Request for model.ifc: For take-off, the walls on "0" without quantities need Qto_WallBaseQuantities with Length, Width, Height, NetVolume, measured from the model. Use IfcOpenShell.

First a look at what the model holds.

```python
import ifcopenshell
import ifcopenshell.util.element
import ifcopenshell.util.unit

model = ifcopenshell.open("model.ifc")
print(model.schema)
for unit_type in ("LENGTHUNIT", "AREAUNIT", "VOLUMEUNIT"):
    print(unit_type, ifcopenshell.util.unit.calculate_unit_scale(model, unit_type))
storey = next(s for s in model.by_type("IfcBuildingStorey") if s.Name == "0")
walls = [e for e in ifcopenshell.util.element.get_decomposition(storey) if e.is_a("IfcWall")]
for e in sorted(walls, key=lambda e: e.id()):
    print(e.id(), e.is_a(), e.Name, list(ifcopenshell.util.element.get_psets(e, qtos_only=True)), sep=" | ")
```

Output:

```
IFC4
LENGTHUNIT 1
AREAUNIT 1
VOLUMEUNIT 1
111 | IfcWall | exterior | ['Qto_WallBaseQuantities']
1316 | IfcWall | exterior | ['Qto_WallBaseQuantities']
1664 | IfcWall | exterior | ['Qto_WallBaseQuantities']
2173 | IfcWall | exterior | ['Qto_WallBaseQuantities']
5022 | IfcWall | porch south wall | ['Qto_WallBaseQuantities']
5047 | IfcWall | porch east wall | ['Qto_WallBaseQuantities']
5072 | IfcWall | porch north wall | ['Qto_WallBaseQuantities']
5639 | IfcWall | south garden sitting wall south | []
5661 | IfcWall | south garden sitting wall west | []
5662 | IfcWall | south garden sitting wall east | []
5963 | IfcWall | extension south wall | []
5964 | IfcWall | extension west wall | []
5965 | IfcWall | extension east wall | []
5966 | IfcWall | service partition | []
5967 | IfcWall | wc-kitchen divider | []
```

```python
import ifcopenshell
import ifcopenshell.api.pset
import ifcopenshell.geom
import ifcopenshell.util.element
import ifcopenshell.util.shape
import ifcopenshell.util.unit

model = ifcopenshell.open("model.ifc")
unit_scale = ifcopenshell.util.unit.calculate_unit_scale(model)
volume_scale = ifcopenshell.util.unit.calculate_unit_scale(model, "VOLUMEUNIT")
settings = ifcopenshell.geom.settings()

storey = next(s for s in model.by_type("IfcBuildingStorey") if s.Name == "0")
walls = [e for e in ifcopenshell.util.element.get_decomposition(storey) if e.is_a("IfcWall")]

for e in sorted(walls, key=lambda e: e.id()):
    if ifcopenshell.util.element.get_psets(e, qtos_only=True, should_inherit=False):
        continue
    # Geometry comes back in metres, in the element's own axes.
    shape = ifcopenshell.geom.create_shape(settings, e)
    values = {
        "Length": ifcopenshell.util.shape.get_x(shape.geometry) / unit_scale,
        "Width": ifcopenshell.util.shape.get_y(shape.geometry) / unit_scale,
        "Height": ifcopenshell.util.shape.get_z(shape.geometry) / unit_scale,
        "NetVolume": ifcopenshell.util.shape.get_volume(shape.geometry) / volume_scale,
    }
    qto = ifcopenshell.api.pset.add_qto(model, product=e, name="Qto_WallBaseQuantities")
    ifcopenshell.api.pset.edit_qto(model, qto=qto, properties=values)
    print(e.id(), {k: round(v, 3) for k, v in values.items()})

model.write("model_rev.ifc")
```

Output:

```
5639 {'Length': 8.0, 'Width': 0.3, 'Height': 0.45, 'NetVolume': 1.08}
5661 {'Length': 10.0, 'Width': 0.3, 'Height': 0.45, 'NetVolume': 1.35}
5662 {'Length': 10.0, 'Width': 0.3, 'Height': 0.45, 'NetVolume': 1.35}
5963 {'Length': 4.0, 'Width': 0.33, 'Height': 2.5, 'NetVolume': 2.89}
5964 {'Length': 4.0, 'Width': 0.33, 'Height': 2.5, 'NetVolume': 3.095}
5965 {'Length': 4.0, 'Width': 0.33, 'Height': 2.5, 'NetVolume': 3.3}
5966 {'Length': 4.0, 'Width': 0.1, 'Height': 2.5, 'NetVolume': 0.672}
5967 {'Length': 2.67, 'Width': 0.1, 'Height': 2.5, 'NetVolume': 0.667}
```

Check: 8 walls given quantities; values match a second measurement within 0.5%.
